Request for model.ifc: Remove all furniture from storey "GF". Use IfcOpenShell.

First a look at what the model holds.

```python
import ifcopenshell
import ifcopenshell.util.element

model = ifcopenshell.open("model.ifc")
print(model.schema)
storey = next(s for s in model.by_type("IfcBuildingStorey") if s.Name == "GF")
furniture = [e for e in ifcopenshell.util.element.get_decomposition(storey) if e.is_a("IfcFurnishingElement")]
seen = {}
for e in furniture:
    element_type = ifcopenshell.util.element.get_type(e)
    name = element_type.Name if element_type not in (None, e) else None
    seen[name] = seen.get(name, 0) + 1
for name, count in sorted(seen.items(), key=str):
    print(count, "x", name)
```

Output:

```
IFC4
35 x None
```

```python
import ifcopenshell
import ifcopenshell.api.root
import ifcopenshell.util.element

model = ifcopenshell.open("model.ifc")

storey = next(s for s in model.by_type("IfcBuildingStorey") if s.Name == "GF")
furniture = [e for e in ifcopenshell.util.element.get_decomposition(storey) if e.is_a("IfcFurnishingElement")]

for e in furniture:
    ifcopenshell.api.root.remove_product(model, product=e)
print(len(furniture), "removed")

model.write("model-out.ifc")
```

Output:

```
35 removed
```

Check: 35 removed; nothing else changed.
